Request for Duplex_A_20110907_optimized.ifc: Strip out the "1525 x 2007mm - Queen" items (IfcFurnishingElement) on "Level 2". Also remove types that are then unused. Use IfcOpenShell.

First a look at what the model holds.

```python
import ifcopenshell
import ifcopenshell.util.element

model = ifcopenshell.open("Duplex_A_20110907_optimized.ifc")
print(model.schema)
storey = next(s for s in model.by_type("IfcBuildingStorey") if s.Name == "Level 2")
furniture = [e for e in ifcopenshell.util.element.get_decomposition(storey) if e.is_a("IfcFurnishingElement")]
seen = {}
for e in furniture:
    element_type = ifcopenshell.util.element.get_type(e)
    name = element_type.Name if element_type not in (None, e) else None
    seen[name] = seen.get(name, 0) + 1
for name, count in sorted(seen.items(), key=str):
    print(count, "x", name)
```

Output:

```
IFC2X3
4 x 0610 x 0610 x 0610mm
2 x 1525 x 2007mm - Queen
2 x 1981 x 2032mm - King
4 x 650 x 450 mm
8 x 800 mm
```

```python
import ifcopenshell
import ifcopenshell.api.root
import ifcopenshell.util.element

model = ifcopenshell.open("Duplex_A_20110907_optimized.ifc")

storey = next(s for s in model.by_type("IfcBuildingStorey") if s.Name == "Level 2")
furniture = [e for e in ifcopenshell.util.element.get_decomposition(storey) if e.is_a("IfcFurnishingElement")]
targets = [e for e in furniture if (t := ifcopenshell.util.element.get_type(e)) not in (None, e) and t.Name == "1525 x 2007mm - Queen"]
types = {ifcopenshell.util.element.get_type(e) for e in targets} - {None, *targets}

for e in targets:
    ifcopenshell.api.root.remove_product(model, product=e)
print(len(targets), "removed")

unused = [t for t in types if not ifcopenshell.util.element.get_types(t)]
for t in unused:
    ifcopenshell.api.root.remove_product(model, product=t)
print(len(unused), "unused types removed")

model.write("Duplex_A_20110907_optimized_rev.ifc")
```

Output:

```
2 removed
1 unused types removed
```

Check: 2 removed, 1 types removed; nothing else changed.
